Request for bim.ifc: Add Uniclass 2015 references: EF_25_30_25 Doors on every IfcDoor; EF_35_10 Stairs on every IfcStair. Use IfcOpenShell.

First a look at what the model holds.

```python
import ifcopenshell

model = ifcopenshell.open("bim.ifc")
print(model.schema)
print("classifications:", [c.Name for c in model.by_type("IfcClassification")])
for ifc_class in ("IfcDoor", "IfcRoof", "IfcStair", "IfcWall", "IfcWindow"):
    print(ifc_class, len(model.by_type(ifc_class)))
```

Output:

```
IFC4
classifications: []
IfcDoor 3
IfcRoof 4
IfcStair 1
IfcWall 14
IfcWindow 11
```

```python
import ifcopenshell
import ifcopenshell.api.classification

model = ifcopenshell.open("bim.ifc")

system = ifcopenshell.api.classification.add_classification(model, classification="Uniclass 2015")

codes = {
    "IfcDoor": ("EF_25_30_25", "Doors"),
    "IfcStair": ("EF_35_10", "Stairs"),
}
for ifc_class, (code, name) in codes.items():
    products = model.by_type(ifc_class)
    ifcopenshell.api.classification.add_reference(
        model, products=products, classification=system, identification=code, name=name
    )
    print(code, len(products))

model.write("bim_updated.ifc")
```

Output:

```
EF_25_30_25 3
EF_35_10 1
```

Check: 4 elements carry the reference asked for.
